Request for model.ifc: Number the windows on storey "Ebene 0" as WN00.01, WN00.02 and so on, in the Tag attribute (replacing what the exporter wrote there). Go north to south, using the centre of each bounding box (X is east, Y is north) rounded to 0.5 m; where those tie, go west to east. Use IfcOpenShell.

First a look at what the model holds.

```python
import ifcopenshell
import ifcopenshell.util.element
import ifcopenshell.util.placement

model = ifcopenshell.open("model.ifc")
print(model.schema)
storey = next(s for s in model.by_type("IfcBuildingStorey") if s.Name == "Ebene 0")
windows = [e for e in ifcopenshell.util.element.get_decomposition(storey) if e.is_a("IfcWindow")]
for e in sorted(windows, key=lambda e: e.id()):
    origin = ifcopenshell.util.placement.get_local_placement(e.ObjectPlacement)[:3, 3]
    print(e.id(), e.Tag, e.Name, origin.round(2) + 0.0, sep=" | ")
```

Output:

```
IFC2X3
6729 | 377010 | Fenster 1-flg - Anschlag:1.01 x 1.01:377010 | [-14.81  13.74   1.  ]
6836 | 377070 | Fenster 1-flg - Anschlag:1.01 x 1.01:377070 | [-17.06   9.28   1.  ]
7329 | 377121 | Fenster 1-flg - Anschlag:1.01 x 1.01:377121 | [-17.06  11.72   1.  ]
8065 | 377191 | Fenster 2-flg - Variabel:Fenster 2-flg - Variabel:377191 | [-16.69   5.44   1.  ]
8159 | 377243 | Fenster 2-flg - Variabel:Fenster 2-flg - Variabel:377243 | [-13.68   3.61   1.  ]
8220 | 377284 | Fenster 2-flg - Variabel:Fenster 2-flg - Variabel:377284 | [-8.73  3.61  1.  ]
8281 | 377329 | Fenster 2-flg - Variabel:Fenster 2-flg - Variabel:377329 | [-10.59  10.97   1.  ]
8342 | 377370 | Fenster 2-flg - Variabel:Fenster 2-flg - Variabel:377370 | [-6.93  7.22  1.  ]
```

```python
import ifcopenshell
import ifcopenshell.geom
import ifcopenshell.util.element
import ifcopenshell.util.shape

model = ifcopenshell.open("model.ifc")
settings = ifcopenshell.geom.settings()
settings.set("use-world-coords", True)


def centre(element):
    shape = ifcopenshell.geom.create_shape(settings, element)
    return ifcopenshell.util.shape.get_bbox_centroid(shape.geometry)


storey = next(s for s in model.by_type("IfcBuildingStorey") if s.Name == "Ebene 0")
windows = [e for e in ifcopenshell.util.element.get_decomposition(storey) if e.is_a("IfcWindow")]

# Insertion points can sit at a corner or the storey origin, so sort by the geometry (in metres).
centres = {e: centre(e) for e in windows}
windows.sort(key=lambda e: (-round(centres[e][1] / 0.5), centres[e][0]))

for i, e in enumerate(windows, start=1):
    number = f"WN00.{i:02d}"
    e.Tag = number
    print(e.id(), number)

model.write("model_rev.ifc")
```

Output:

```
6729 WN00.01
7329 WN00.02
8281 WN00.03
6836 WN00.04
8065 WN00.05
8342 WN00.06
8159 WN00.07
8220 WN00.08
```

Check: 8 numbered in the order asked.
